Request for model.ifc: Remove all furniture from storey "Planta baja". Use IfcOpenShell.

First a look at what the model holds.

```python
import ifcopenshell
import ifcopenshell.util.element

model = ifcopenshell.open("model.ifc")
print(model.schema)
storey = next(s for s in model.by_type("IfcBuildingStorey") if s.Name == "Planta baja")
furniture = [e for e in ifcopenshell.util.element.get_decomposition(storey) if e.is_a("IfcFurnishingElement")]
seen = {}
for e in furniture:
    element_type = ifcopenshell.util.element.get_type(e)
    name = element_type.Name if element_type not in (None, e) else None
    seen[name] = seen.get(name, 0) + 1
for name, count in sorted(seen.items(), key=str):
    print(count, "x", name)
```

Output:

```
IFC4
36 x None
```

```python
import ifcopenshell
import ifcopenshell.api.root
import ifcopenshell.util.element

model = ifcopenshell.open("model.ifc")

storey = next(s for s in model.by_type("IfcBuildingStorey") if s.Name == "Planta baja")
furniture = [e for e in ifcopenshell.util.element.get_decomposition(storey) if e.is_a("IfcFurnishingElement")]

for e in furniture:
    ifcopenshell.api.root.remove_product(model, product=e)
print(len(furniture), "removed")

model.write("model_updated.ifc")
```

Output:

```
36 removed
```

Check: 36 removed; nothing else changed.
